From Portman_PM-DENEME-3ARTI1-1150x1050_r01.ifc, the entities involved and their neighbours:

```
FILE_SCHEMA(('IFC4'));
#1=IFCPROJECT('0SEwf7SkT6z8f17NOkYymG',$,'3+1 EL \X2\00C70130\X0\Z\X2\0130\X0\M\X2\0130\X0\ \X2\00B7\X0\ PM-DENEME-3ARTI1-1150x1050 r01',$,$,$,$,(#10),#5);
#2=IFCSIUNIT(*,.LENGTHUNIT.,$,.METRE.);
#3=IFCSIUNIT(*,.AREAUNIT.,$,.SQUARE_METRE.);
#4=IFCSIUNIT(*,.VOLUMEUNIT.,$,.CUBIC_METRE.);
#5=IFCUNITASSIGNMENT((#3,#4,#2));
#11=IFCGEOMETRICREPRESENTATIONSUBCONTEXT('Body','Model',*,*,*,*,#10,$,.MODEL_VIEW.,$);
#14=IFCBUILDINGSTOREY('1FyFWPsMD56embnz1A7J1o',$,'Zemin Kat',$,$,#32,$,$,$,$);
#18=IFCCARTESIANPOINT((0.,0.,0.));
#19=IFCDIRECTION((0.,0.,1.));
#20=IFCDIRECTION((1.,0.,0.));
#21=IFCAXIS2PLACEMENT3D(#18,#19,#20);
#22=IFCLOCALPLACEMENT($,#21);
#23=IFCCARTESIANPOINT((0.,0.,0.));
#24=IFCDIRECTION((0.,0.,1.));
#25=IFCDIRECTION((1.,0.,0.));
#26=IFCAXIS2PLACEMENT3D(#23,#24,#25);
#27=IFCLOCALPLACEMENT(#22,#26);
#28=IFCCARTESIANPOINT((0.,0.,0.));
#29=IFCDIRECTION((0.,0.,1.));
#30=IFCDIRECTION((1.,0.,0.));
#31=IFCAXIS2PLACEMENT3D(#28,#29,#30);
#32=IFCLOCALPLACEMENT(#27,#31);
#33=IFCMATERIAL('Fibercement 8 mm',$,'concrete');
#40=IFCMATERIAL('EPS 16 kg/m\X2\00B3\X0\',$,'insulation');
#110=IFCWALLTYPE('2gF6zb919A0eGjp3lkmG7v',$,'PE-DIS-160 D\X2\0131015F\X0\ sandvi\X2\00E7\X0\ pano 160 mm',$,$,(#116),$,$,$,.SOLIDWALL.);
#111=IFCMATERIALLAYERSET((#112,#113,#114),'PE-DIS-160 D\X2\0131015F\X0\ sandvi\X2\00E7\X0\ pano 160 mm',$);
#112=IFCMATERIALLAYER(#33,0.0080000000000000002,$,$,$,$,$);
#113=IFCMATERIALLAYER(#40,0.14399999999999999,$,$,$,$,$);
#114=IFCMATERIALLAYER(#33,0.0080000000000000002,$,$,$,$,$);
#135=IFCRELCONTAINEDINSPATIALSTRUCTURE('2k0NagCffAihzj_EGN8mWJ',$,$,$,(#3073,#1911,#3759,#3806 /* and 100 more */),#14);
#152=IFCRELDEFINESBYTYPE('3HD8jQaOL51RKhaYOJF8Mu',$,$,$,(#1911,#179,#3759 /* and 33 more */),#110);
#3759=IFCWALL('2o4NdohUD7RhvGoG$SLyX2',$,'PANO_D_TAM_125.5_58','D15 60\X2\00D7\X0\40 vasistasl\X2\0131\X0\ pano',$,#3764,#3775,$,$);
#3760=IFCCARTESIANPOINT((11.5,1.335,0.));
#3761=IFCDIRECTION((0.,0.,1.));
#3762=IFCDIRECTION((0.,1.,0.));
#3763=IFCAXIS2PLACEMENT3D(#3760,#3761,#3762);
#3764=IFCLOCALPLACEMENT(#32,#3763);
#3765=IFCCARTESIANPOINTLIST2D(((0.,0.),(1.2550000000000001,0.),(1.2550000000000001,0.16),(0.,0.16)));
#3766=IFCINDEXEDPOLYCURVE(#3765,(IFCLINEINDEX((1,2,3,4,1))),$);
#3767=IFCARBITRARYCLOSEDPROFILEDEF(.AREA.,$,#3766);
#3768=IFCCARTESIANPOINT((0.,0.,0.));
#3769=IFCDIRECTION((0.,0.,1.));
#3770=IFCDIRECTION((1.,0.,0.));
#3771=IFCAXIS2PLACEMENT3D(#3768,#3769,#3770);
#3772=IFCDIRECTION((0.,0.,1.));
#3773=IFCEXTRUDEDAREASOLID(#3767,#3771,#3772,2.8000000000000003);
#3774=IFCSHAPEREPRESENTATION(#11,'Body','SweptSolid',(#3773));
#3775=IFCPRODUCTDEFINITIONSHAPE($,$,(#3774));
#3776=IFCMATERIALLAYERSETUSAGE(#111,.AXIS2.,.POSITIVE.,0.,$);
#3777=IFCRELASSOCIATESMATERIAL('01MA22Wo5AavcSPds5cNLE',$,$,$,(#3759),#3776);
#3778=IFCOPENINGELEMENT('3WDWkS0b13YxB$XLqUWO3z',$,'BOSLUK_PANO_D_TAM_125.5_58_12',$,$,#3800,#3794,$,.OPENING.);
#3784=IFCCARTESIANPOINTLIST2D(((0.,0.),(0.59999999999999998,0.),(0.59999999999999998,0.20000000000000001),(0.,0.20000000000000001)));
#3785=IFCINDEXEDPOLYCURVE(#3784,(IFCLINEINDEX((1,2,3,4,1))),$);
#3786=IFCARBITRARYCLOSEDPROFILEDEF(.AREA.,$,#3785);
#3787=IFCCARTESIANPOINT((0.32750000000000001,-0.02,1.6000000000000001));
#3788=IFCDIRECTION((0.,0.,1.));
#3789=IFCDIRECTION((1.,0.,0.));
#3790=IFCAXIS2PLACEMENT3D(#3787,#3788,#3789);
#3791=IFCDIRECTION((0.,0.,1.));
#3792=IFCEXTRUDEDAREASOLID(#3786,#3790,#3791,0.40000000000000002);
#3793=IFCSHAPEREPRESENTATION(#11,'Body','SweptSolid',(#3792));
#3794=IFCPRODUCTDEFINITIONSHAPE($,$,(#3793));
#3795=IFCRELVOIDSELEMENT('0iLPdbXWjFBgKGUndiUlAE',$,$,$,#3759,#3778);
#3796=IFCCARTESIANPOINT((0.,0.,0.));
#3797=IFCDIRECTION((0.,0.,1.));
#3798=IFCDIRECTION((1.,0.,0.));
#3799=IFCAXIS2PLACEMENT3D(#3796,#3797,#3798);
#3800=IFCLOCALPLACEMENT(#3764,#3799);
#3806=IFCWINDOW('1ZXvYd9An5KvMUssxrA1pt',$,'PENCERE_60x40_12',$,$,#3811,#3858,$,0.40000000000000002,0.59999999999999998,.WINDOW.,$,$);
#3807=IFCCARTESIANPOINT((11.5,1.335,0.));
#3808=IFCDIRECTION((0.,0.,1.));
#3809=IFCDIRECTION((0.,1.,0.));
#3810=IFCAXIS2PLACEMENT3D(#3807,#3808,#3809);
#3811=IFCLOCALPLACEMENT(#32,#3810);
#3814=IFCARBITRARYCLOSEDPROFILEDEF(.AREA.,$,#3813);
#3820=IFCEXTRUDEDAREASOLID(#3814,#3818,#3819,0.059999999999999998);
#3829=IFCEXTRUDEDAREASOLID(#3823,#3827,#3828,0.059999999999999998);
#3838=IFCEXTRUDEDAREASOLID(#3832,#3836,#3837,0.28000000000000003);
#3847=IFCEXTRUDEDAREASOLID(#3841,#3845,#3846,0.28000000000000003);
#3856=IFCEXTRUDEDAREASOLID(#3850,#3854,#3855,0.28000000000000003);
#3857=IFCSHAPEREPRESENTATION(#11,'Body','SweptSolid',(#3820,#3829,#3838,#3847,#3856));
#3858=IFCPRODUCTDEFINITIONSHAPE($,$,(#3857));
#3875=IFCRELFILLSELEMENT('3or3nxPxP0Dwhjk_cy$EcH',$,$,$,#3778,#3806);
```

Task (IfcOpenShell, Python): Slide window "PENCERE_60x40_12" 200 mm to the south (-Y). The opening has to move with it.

```python
import ifcopenshell
import ifcopenshell.api.geometry
import ifcopenshell.util.placement
import ifcopenshell.util.unit

model = ifcopenshell.open("Portman_PM-DENEME-3ARTI1-1150x1050_r01.ifc")
unit_scale = ifcopenshell.util.unit.calculate_unit_scale(model)

window = model.by_id(3806)
opening = window.FillsVoids[0].RelatingOpeningElement
wall = opening.VoidsElements[0].RelatingBuildingElement

wall_matrix = ifcopenshell.util.placement.get_local_placement(wall.ObjectPlacement)
shift = wall_matrix[:3, 0] * -0.2 / unit_scale
before = ifcopenshell.util.placement.get_local_placement(window.ObjectPlacement)[:3, 3].copy()

# The window is not placed relative to its opening, so move both.
for product in (opening, window):
    matrix = ifcopenshell.util.placement.get_local_placement(product.ObjectPlacement)
    matrix[:3, 3] += shift
    ifcopenshell.api.geometry.edit_object_placement(model, product=product, matrix=matrix, is_si=False)

after = ifcopenshell.util.placement.get_local_placement(window.ObjectPlacement)[:3, 3]
print("window moved by", (after - before).round(3) + 0.0)

model.write("Portman_PM-DENEME-3ARTI1-1150x1050_r01_edited.ifc")
```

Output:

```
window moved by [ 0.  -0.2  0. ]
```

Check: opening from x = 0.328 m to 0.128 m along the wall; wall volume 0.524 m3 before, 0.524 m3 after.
